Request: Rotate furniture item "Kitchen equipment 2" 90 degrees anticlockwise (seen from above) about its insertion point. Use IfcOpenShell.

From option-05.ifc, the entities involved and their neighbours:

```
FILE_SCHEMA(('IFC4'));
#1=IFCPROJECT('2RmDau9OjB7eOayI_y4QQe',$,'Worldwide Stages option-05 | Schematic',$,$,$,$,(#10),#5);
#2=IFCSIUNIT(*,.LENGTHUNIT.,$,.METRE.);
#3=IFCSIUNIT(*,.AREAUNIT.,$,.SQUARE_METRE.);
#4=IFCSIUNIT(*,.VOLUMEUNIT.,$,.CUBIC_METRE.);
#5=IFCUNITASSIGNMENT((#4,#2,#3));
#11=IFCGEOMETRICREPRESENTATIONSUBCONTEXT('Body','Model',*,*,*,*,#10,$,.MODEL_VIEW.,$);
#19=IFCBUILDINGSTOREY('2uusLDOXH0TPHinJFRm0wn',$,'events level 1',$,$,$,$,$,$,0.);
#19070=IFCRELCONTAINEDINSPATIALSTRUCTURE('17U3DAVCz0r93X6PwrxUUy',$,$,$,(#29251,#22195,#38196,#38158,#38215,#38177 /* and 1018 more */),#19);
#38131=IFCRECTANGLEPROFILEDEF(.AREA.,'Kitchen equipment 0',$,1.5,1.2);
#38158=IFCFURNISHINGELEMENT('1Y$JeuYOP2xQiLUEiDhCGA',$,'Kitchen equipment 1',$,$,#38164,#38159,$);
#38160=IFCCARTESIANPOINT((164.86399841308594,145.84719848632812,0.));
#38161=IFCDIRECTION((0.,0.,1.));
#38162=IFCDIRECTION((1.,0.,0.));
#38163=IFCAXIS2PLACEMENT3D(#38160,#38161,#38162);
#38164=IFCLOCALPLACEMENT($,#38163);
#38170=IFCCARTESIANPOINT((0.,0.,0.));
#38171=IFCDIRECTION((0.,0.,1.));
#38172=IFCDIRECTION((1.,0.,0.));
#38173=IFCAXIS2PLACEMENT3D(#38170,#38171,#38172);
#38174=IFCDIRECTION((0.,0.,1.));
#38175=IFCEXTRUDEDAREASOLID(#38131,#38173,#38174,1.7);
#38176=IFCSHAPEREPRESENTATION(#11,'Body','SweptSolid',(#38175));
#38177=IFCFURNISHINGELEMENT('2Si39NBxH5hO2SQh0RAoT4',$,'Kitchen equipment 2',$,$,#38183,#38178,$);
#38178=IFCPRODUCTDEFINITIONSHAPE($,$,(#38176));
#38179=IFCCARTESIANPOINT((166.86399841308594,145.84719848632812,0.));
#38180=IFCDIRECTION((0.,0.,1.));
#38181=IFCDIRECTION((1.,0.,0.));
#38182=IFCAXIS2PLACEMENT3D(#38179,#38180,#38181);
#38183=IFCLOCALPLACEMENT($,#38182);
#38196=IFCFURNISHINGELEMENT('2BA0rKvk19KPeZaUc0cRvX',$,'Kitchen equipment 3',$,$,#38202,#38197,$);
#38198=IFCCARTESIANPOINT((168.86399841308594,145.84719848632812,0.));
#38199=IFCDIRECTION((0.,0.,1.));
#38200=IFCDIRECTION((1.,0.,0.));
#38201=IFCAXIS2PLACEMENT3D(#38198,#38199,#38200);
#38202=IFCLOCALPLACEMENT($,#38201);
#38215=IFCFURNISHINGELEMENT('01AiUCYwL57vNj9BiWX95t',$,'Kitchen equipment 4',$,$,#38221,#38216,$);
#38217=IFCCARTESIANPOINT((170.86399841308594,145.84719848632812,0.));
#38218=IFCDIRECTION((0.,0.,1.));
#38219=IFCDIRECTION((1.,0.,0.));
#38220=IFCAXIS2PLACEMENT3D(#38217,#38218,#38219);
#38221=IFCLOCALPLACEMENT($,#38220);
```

```python
import ifcopenshell
import ifcopenshell.api.geometry
import ifcopenshell.util.placement

model = ifcopenshell.open("option-05.ifc")

item = model.by_guid("2Si39NBxH5hO2SQh0RAoT4")
matrix = ifcopenshell.util.placement.get_local_placement(item.ObjectPlacement)
matrix = matrix @ ifcopenshell.util.placement.rotation(90, "Z")
ifcopenshell.api.geometry.edit_object_placement(model, product=item, matrix=matrix, is_si=False)

print(ifcopenshell.util.placement.get_local_placement(item.ObjectPlacement).round(3) + 0.0)

model.write("option-05_edited.ifc")
```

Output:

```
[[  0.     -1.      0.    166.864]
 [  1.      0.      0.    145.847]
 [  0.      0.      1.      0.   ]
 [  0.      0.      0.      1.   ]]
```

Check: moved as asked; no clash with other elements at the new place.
